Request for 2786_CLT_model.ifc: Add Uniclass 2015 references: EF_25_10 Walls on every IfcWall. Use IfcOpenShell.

First a look at what the model holds.

```python
import ifcopenshell

model = ifcopenshell.open("2786_CLT_model.ifc")
print(model.schema)
print("classifications:", [c.Name for c in model.by_type("IfcClassification")])
for ifc_class in ("IfcDoor", "IfcRoof", "IfcStair", "IfcWall", "IfcWindow"):
    print(ifc_class, len(model.by_type(ifc_class)))
```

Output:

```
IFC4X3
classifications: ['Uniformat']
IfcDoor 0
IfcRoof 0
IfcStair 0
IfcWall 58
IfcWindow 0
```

```python
import ifcopenshell
import ifcopenshell.api.classification

model = ifcopenshell.open("2786_CLT_model.ifc")

system = ifcopenshell.api.classification.add_classification(model, classification="Uniclass 2015")

codes = {
    "IfcWall": ("EF_25_10", "Walls"),
}
for ifc_class, (code, name) in codes.items():
    products = model.by_type(ifc_class)
    ifcopenshell.api.classification.add_reference(
        model, products=products, classification=system, identification=code, name=name
    )
    print(code, len(products))

model.write("2786_CLT_model_updated.ifc")
```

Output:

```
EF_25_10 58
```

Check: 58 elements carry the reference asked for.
